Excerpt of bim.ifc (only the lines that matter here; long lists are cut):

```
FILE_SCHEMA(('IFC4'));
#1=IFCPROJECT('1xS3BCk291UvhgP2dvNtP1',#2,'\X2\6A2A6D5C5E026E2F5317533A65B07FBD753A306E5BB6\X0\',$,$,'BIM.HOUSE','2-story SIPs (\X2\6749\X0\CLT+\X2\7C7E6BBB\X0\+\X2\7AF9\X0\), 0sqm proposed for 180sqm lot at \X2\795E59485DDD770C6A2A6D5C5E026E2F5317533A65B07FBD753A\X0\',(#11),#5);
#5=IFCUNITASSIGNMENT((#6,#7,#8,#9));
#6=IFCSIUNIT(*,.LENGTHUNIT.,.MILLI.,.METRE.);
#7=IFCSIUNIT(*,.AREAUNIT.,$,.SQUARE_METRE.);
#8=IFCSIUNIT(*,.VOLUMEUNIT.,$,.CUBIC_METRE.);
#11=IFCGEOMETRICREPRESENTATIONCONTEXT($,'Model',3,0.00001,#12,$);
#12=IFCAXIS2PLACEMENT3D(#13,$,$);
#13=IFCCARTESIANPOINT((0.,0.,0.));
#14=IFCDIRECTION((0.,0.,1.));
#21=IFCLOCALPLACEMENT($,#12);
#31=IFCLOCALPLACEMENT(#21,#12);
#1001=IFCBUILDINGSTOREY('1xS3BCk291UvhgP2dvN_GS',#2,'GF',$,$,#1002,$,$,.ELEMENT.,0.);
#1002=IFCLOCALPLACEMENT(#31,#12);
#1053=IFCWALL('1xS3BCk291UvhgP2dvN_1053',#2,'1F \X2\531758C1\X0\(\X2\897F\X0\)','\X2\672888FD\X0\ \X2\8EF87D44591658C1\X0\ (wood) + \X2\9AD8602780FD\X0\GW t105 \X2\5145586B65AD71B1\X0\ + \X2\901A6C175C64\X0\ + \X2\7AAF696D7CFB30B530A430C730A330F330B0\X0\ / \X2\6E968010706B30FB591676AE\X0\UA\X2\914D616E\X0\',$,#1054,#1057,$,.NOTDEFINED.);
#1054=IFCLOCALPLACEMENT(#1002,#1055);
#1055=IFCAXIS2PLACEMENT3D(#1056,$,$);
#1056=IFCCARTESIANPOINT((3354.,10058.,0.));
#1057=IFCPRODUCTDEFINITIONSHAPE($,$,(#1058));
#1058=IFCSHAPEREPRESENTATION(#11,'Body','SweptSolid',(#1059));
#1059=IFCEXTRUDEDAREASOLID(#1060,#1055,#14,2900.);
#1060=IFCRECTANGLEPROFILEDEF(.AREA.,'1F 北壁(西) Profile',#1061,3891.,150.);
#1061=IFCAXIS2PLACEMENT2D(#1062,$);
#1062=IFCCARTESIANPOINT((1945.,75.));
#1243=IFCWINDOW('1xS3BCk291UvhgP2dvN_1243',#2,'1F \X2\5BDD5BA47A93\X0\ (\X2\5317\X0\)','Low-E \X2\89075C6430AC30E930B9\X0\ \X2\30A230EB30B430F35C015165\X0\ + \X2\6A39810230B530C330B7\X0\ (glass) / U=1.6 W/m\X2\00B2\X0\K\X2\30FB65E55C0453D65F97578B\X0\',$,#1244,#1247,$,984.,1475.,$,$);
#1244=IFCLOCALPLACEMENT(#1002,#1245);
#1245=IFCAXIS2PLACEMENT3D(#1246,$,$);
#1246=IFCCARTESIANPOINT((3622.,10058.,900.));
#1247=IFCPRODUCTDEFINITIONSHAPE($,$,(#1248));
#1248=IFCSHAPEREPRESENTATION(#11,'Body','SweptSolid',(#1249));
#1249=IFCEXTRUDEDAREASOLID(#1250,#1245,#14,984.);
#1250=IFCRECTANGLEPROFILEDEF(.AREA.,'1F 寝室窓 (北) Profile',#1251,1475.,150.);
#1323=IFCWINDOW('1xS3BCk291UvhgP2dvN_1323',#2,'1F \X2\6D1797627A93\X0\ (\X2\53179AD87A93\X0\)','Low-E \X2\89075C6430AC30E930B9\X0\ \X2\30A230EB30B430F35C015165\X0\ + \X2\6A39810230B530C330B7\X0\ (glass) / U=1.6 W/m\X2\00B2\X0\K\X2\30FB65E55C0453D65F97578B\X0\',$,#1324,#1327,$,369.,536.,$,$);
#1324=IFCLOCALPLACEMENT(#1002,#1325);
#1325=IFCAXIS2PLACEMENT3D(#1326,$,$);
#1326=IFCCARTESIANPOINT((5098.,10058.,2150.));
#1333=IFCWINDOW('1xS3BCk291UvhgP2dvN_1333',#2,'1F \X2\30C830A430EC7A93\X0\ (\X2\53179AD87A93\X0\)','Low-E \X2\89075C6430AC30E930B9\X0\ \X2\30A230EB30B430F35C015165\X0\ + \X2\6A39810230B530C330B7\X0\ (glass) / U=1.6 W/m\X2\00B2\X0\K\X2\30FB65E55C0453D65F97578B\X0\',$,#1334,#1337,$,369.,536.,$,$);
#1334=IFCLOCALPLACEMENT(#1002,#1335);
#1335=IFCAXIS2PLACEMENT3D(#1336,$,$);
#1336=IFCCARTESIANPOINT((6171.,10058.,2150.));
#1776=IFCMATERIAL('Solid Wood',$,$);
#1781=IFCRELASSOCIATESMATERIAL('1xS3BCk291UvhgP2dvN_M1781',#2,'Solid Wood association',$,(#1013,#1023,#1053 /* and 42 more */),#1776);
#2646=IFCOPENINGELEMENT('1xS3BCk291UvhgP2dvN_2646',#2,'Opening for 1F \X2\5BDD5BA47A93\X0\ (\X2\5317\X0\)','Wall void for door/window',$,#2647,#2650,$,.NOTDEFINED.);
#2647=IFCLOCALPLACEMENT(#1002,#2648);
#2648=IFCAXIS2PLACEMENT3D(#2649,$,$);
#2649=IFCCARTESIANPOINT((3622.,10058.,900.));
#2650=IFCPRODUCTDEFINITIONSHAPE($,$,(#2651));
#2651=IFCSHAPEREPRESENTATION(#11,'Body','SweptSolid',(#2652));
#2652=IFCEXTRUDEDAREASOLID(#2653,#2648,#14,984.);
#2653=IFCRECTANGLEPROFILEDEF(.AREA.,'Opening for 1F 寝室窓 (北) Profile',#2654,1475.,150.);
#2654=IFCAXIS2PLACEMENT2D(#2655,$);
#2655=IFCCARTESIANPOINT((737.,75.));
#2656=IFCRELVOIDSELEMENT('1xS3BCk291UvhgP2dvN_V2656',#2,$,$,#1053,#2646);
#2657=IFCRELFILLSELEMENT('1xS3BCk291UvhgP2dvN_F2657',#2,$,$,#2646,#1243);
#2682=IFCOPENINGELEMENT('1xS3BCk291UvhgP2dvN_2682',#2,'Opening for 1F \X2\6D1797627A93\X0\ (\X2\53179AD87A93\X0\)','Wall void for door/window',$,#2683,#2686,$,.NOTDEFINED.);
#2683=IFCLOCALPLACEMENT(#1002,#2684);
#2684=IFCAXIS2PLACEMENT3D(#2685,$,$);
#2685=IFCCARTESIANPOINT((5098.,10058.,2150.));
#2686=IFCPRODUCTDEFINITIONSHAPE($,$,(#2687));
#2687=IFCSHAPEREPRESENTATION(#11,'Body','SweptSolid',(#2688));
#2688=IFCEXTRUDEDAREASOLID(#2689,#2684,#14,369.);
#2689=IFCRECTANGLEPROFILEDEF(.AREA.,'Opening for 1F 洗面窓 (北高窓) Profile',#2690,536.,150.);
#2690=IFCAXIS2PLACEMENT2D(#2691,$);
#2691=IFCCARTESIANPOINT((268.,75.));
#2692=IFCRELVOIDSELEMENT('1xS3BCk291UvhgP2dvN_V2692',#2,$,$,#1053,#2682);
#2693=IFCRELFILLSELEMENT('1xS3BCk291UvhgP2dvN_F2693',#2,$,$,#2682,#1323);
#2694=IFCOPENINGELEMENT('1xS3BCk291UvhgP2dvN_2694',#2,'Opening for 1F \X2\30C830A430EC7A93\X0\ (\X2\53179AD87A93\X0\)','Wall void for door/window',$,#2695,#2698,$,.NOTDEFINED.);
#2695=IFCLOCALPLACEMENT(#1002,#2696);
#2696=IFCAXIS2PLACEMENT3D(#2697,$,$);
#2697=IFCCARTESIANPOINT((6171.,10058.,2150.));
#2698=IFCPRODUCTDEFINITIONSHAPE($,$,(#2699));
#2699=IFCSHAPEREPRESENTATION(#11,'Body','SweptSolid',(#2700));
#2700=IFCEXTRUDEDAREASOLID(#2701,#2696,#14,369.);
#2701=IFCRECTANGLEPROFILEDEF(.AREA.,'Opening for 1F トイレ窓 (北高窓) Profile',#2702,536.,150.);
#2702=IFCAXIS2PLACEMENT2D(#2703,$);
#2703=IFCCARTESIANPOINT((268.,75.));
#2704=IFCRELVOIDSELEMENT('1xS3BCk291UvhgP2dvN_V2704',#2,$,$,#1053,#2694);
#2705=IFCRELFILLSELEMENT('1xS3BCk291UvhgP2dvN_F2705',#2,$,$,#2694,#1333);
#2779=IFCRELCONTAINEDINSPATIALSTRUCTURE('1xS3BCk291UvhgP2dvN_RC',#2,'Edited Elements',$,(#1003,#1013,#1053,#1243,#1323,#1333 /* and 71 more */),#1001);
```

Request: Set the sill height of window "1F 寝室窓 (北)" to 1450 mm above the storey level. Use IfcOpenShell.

```python
import numpy as np
import ifcopenshell
import ifcopenshell.api.geometry
import ifcopenshell.geom
import ifcopenshell.util.element
import ifcopenshell.util.placement
import ifcopenshell.util.shape
import ifcopenshell.util.unit

model = ifcopenshell.open("bim.ifc")
unit_scale = ifcopenshell.util.unit.calculate_unit_scale(model)

window = model.by_guid("1xS3BCk291UvhgP2dvN_1243")
opening = window.FillsVoids[0].RelatingOpeningElement
storey = ifcopenshell.util.element.get_container(window, ifc_class="IfcBuildingStorey")
level = ifcopenshell.util.placement.get_local_placement(storey.ObjectPlacement)[2, 3]

# The opening's origin need not be at the sill, so measure its lowest point.
shape = ifcopenshell.geom.create_shape(ifcopenshell.geom.settings(), opening)
bottom = ifcopenshell.util.shape.get_shape_bottom_elevation(shape, shape.geometry) / unit_scale
dz = level + 1.45 / unit_scale - bottom

shift = np.array([0.0, 0.0, dz])
# The window is not placed relative to its opening, so move both.
for product in (opening, window):
    matrix = ifcopenshell.util.placement.get_local_placement(product.ObjectPlacement)
    matrix[:3, 3] += shift
    ifcopenshell.api.geometry.edit_object_placement(model, product=product, matrix=matrix, is_si=False)

print(f"moved by {dz * unit_scale:+.3f} m")

model.write("bim-out.ifc")
```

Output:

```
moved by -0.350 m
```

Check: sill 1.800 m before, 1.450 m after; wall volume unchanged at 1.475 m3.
